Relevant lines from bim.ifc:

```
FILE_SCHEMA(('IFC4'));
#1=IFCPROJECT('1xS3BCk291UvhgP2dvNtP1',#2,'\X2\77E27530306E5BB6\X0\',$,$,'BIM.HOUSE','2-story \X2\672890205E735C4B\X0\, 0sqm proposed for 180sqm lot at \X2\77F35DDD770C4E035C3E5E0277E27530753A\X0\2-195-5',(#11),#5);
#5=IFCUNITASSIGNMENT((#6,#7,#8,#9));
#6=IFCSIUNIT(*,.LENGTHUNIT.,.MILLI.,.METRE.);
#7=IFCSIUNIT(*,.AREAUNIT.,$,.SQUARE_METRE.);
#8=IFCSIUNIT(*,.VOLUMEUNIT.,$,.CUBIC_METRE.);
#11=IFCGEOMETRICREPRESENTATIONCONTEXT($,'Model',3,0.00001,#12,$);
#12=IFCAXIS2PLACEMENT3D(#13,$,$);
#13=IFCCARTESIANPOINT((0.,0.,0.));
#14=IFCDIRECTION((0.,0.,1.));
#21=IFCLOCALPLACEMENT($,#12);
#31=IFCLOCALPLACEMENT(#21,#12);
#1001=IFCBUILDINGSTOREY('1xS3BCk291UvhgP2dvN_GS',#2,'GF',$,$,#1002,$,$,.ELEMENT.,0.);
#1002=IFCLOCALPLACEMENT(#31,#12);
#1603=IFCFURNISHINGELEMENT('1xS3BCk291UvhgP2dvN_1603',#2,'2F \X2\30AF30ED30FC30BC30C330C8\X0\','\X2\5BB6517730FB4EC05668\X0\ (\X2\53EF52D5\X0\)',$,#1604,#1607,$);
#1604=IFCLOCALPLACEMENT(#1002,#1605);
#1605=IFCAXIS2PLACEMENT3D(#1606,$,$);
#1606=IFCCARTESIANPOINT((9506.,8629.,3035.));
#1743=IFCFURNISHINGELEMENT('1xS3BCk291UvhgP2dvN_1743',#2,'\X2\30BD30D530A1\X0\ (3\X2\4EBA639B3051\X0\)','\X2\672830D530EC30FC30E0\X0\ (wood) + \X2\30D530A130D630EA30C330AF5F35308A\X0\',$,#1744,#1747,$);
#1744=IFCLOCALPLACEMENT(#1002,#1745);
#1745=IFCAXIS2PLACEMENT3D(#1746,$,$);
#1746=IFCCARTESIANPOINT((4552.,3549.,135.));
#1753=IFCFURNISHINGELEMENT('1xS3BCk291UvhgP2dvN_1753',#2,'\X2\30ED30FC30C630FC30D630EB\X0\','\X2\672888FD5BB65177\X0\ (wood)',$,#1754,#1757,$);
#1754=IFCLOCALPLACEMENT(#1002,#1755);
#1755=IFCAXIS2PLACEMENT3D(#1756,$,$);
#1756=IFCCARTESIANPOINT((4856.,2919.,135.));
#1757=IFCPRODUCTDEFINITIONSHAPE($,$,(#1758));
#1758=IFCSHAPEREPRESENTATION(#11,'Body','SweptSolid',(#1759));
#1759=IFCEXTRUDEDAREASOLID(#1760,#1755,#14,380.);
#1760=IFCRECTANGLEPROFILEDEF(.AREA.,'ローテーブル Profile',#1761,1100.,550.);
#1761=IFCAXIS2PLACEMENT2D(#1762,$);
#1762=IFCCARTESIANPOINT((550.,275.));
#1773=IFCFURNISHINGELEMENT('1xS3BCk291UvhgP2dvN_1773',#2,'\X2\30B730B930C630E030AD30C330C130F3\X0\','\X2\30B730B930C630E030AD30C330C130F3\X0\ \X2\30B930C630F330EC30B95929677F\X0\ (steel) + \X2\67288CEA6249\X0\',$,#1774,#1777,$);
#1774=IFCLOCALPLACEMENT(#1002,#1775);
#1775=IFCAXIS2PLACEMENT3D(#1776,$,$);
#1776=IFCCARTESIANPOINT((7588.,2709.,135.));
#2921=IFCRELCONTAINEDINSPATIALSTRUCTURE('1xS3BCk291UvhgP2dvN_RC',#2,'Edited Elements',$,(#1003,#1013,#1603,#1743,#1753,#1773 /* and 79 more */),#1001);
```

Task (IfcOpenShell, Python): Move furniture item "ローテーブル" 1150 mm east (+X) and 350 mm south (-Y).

```python
import ifcopenshell
import ifcopenshell.api.geometry
import ifcopenshell.util.placement
import ifcopenshell.util.unit

model = ifcopenshell.open("bim.ifc")
unit_scale = ifcopenshell.util.unit.calculate_unit_scale(model)

item = model.by_id(1753)
matrix = ifcopenshell.util.placement.get_local_placement(item.ObjectPlacement)
matrix[0, 3] += 1.15 / unit_scale
matrix[1, 3] -= 0.35 / unit_scale
ifcopenshell.api.geometry.edit_object_placement(model, product=item, matrix=matrix, is_si=False)

print(ifcopenshell.util.placement.get_local_placement(item.ObjectPlacement).round(3) + 0.0)

model.write("bim_edited.ifc")
```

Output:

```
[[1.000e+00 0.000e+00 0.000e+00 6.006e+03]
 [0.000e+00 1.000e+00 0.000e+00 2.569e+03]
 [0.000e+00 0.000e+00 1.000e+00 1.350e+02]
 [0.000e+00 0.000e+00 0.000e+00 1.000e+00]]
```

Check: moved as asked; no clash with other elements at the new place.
